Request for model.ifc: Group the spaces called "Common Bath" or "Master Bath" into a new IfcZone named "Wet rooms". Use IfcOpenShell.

First a look at what the model holds.

```python
import ifcopenshell

model = ifcopenshell.open("model.ifc")
print(model.schema)
seen = {}
for space in model.by_type("IfcSpace"):
    seen[space.LongName] = seen.get(space.LongName, 0) + 1
for name, count in sorted(seen.items(), key=str):
    print(count, "x", name)
print("zones:", [z.Name for z in model.by_type("IfcZone")][:20])
```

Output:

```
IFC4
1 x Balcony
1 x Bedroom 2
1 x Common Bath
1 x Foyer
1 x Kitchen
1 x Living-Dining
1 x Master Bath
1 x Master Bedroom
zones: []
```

```python
import ifcopenshell
import ifcopenshell.api.group
import ifcopenshell.api.root

model = ifcopenshell.open("model.ifc")

names = {"Common Bath", "Master Bath"}
spaces = [s for s in model.by_type("IfcSpace") if s.LongName in names]

zone = ifcopenshell.api.root.create_entity(model, ifc_class="IfcZone", name="Wet rooms")
ifcopenshell.api.group.assign_group(model, products=spaces, group=zone)
print(len(spaces), "spaces in", zone.Name)

model.write("model_rev.ifc")
```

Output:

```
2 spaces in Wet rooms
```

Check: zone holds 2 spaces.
